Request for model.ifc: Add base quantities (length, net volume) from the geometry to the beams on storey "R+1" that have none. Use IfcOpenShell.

First a look at what the model holds.

```python
import ifcopenshell
import ifcopenshell.util.element
import ifcopenshell.util.unit

model = ifcopenshell.open("model.ifc")
print(model.schema)
for unit_type in ("LENGTHUNIT", "AREAUNIT", "VOLUMEUNIT"):
    print(unit_type, ifcopenshell.util.unit.calculate_unit_scale(model, unit_type))
storey = next(s for s in model.by_type("IfcBuildingStorey") if s.Name == "R+1")
beams = [e for e in ifcopenshell.util.element.get_decomposition(storey) if e.is_a("IfcBeam")]
for e in sorted(beams, key=lambda e: e.id()):
    print(e.id(), e.is_a(), e.Name, list(ifcopenshell.util.element.get_psets(e, qtos_only=True)), sep=" | ")
```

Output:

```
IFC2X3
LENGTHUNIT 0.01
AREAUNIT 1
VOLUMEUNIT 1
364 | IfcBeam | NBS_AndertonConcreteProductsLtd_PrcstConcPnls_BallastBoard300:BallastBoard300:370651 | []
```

```python
import ifcopenshell
import ifcopenshell.api.pset
import ifcopenshell.geom
import ifcopenshell.util.element
import ifcopenshell.util.shape
import ifcopenshell.util.unit

model = ifcopenshell.open("model.ifc")
unit_scale = ifcopenshell.util.unit.calculate_unit_scale(model)
volume_scale = ifcopenshell.util.unit.calculate_unit_scale(model, "VOLUMEUNIT")
settings = ifcopenshell.geom.settings()

storey = next(s for s in model.by_type("IfcBuildingStorey") if s.Name == "R+1")
beams = [e for e in ifcopenshell.util.element.get_decomposition(storey) if e.is_a("IfcBeam")]

for e in sorted(beams, key=lambda e: e.id()):
    if ifcopenshell.util.element.get_psets(e, qtos_only=True, should_inherit=False):
        continue
    # Geometry comes back in metres, in the element's own axes.
    shape = ifcopenshell.geom.create_shape(settings, e)
    values = {
        "Length": ifcopenshell.util.shape.get_max_xyz(shape.geometry) / unit_scale,
        "NetVolume": ifcopenshell.util.shape.get_volume(shape.geometry) / volume_scale,
    }
    qto = ifcopenshell.api.pset.add_qto(model, product=e, name="BaseQuantities")
    ifcopenshell.api.pset.edit_qto(model, qto=qto, properties=values)
    print(e.id(), {k: round(v, 3) for k, v in values.items()})

model.write("model-out.ifc")
```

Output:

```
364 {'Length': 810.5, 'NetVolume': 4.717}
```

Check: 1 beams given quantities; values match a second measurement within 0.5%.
